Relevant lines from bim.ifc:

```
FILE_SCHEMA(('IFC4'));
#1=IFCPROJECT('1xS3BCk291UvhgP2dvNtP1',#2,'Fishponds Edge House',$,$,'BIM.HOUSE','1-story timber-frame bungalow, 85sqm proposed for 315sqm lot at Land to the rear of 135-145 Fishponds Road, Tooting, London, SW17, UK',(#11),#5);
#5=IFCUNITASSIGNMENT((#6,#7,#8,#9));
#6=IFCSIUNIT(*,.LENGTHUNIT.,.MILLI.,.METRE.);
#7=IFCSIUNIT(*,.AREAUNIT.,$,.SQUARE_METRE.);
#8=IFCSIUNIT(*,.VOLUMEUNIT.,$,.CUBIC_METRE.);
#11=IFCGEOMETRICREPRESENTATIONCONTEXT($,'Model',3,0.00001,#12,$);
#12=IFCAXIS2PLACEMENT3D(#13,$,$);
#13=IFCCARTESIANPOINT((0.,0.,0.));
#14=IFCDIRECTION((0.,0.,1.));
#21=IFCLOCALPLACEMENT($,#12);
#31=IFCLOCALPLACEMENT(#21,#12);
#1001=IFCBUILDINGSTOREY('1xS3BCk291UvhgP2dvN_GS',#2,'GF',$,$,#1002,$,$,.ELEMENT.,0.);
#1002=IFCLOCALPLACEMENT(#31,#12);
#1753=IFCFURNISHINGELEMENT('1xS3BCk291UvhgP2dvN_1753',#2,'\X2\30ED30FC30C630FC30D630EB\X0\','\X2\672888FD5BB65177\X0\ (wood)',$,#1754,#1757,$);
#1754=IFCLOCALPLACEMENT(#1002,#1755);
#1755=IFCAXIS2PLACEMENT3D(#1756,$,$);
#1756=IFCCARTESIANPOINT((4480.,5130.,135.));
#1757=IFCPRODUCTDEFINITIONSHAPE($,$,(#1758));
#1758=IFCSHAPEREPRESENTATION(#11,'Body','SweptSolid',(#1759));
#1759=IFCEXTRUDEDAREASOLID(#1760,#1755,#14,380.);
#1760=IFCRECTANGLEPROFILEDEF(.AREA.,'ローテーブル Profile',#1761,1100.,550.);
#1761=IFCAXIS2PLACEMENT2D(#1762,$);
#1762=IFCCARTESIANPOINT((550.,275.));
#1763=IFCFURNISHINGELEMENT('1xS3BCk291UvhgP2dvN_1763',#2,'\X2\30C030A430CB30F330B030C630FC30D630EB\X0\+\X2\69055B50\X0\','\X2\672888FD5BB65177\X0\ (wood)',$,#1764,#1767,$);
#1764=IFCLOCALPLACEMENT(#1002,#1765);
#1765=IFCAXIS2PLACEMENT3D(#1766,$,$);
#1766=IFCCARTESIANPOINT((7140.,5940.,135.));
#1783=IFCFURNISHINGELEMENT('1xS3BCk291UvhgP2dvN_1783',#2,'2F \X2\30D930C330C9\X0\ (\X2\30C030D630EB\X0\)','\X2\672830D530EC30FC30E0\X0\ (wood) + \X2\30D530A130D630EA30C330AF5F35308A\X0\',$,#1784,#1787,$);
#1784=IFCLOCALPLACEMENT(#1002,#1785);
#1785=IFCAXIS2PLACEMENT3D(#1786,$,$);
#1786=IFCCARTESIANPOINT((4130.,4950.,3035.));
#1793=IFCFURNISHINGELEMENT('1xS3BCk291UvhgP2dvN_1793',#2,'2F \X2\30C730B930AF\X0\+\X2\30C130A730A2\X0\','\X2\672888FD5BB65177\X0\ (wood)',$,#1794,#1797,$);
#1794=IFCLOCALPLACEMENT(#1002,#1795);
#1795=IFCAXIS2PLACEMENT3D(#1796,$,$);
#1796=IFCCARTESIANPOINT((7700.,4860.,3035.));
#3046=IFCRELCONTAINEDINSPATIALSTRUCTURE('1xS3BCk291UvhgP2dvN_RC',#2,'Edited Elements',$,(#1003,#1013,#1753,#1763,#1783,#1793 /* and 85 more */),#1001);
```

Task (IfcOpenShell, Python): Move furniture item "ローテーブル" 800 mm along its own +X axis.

```python
import ifcopenshell
import ifcopenshell.api.geometry
import ifcopenshell.util.placement
import ifcopenshell.util.unit

model = ifcopenshell.open("bim.ifc")
unit_scale = ifcopenshell.util.unit.calculate_unit_scale(model)

item = model.by_guid("1xS3BCk291UvhgP2dvN_1753")
matrix = ifcopenshell.util.placement.get_local_placement(item.ObjectPlacement)
matrix[:3, 3] += matrix[:3, 0] * 0.8 / unit_scale
ifcopenshell.api.geometry.edit_object_placement(model, product=item, matrix=matrix, is_si=False)

print(ifcopenshell.util.placement.get_local_placement(item.ObjectPlacement).round(3) + 0.0)

model.write("bim-out.ifc")
```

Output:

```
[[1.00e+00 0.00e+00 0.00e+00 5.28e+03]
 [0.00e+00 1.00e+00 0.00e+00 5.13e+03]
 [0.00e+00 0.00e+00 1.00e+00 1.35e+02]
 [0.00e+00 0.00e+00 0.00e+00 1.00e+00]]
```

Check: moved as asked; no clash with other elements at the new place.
